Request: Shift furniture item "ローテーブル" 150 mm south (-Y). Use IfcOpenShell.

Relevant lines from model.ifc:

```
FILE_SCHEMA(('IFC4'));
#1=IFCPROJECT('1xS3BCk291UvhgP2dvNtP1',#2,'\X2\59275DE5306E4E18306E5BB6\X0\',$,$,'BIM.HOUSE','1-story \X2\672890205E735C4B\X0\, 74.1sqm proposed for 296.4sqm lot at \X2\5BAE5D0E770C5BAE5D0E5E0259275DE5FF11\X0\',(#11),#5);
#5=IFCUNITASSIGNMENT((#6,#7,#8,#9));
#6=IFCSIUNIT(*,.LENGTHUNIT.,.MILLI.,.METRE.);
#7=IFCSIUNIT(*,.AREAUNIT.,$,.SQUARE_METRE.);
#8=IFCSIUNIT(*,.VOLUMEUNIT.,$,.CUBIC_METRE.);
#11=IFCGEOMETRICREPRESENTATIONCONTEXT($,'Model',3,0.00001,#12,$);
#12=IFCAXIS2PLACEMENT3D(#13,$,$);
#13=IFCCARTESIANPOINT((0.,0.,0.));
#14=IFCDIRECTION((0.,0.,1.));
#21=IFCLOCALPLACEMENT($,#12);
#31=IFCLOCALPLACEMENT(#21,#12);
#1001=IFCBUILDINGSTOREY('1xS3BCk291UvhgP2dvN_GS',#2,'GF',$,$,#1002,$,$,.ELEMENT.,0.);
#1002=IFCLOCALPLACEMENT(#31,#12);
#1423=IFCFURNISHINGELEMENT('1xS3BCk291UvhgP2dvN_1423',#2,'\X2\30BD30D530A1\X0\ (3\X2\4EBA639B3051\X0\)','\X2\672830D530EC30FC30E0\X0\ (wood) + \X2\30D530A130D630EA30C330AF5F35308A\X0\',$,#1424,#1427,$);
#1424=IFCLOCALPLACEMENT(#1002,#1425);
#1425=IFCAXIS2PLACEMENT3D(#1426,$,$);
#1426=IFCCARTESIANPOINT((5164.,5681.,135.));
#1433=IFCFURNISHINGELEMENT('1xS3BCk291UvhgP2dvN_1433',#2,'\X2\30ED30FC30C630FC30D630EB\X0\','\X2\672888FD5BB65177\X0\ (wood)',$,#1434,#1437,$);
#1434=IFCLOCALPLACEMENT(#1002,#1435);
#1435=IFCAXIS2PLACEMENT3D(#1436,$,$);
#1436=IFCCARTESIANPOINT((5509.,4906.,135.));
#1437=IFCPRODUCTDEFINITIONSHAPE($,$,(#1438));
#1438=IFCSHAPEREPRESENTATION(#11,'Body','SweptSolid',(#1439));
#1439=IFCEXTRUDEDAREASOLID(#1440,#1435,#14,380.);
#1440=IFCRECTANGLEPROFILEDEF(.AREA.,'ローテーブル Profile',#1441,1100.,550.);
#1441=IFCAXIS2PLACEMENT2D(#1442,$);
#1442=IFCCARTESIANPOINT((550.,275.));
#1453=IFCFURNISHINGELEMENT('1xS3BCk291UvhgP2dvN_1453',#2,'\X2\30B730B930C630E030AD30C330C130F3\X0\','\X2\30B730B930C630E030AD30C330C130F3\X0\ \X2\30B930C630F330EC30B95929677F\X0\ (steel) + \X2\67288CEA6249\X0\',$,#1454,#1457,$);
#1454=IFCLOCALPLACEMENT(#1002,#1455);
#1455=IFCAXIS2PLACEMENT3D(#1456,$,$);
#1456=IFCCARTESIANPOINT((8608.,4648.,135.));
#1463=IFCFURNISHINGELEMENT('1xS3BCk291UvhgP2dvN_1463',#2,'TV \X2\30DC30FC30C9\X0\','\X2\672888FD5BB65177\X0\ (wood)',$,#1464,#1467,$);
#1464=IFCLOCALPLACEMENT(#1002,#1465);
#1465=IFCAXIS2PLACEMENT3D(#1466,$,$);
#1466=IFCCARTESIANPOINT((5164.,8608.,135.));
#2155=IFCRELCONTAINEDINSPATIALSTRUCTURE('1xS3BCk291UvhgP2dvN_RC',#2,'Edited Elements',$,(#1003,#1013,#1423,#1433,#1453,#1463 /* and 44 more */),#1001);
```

```python
import ifcopenshell
import ifcopenshell.api.geometry
import ifcopenshell.util.placement

model = ifcopenshell.open("model.ifc")

item = model.by_id(1433)
matrix = ifcopenshell.util.placement.get_local_placement(item.ObjectPlacement)
matrix[1, 3] -= 150.0
ifcopenshell.api.geometry.edit_object_placement(model, product=item, matrix=matrix, is_si=False)

print(ifcopenshell.util.placement.get_local_placement(item.ObjectPlacement).round(3) + 0.0)

model.write("model_updated.ifc")
```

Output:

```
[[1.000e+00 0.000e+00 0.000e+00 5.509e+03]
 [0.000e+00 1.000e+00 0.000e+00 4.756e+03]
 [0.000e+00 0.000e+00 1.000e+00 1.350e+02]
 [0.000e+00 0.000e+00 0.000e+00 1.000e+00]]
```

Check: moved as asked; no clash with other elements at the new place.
